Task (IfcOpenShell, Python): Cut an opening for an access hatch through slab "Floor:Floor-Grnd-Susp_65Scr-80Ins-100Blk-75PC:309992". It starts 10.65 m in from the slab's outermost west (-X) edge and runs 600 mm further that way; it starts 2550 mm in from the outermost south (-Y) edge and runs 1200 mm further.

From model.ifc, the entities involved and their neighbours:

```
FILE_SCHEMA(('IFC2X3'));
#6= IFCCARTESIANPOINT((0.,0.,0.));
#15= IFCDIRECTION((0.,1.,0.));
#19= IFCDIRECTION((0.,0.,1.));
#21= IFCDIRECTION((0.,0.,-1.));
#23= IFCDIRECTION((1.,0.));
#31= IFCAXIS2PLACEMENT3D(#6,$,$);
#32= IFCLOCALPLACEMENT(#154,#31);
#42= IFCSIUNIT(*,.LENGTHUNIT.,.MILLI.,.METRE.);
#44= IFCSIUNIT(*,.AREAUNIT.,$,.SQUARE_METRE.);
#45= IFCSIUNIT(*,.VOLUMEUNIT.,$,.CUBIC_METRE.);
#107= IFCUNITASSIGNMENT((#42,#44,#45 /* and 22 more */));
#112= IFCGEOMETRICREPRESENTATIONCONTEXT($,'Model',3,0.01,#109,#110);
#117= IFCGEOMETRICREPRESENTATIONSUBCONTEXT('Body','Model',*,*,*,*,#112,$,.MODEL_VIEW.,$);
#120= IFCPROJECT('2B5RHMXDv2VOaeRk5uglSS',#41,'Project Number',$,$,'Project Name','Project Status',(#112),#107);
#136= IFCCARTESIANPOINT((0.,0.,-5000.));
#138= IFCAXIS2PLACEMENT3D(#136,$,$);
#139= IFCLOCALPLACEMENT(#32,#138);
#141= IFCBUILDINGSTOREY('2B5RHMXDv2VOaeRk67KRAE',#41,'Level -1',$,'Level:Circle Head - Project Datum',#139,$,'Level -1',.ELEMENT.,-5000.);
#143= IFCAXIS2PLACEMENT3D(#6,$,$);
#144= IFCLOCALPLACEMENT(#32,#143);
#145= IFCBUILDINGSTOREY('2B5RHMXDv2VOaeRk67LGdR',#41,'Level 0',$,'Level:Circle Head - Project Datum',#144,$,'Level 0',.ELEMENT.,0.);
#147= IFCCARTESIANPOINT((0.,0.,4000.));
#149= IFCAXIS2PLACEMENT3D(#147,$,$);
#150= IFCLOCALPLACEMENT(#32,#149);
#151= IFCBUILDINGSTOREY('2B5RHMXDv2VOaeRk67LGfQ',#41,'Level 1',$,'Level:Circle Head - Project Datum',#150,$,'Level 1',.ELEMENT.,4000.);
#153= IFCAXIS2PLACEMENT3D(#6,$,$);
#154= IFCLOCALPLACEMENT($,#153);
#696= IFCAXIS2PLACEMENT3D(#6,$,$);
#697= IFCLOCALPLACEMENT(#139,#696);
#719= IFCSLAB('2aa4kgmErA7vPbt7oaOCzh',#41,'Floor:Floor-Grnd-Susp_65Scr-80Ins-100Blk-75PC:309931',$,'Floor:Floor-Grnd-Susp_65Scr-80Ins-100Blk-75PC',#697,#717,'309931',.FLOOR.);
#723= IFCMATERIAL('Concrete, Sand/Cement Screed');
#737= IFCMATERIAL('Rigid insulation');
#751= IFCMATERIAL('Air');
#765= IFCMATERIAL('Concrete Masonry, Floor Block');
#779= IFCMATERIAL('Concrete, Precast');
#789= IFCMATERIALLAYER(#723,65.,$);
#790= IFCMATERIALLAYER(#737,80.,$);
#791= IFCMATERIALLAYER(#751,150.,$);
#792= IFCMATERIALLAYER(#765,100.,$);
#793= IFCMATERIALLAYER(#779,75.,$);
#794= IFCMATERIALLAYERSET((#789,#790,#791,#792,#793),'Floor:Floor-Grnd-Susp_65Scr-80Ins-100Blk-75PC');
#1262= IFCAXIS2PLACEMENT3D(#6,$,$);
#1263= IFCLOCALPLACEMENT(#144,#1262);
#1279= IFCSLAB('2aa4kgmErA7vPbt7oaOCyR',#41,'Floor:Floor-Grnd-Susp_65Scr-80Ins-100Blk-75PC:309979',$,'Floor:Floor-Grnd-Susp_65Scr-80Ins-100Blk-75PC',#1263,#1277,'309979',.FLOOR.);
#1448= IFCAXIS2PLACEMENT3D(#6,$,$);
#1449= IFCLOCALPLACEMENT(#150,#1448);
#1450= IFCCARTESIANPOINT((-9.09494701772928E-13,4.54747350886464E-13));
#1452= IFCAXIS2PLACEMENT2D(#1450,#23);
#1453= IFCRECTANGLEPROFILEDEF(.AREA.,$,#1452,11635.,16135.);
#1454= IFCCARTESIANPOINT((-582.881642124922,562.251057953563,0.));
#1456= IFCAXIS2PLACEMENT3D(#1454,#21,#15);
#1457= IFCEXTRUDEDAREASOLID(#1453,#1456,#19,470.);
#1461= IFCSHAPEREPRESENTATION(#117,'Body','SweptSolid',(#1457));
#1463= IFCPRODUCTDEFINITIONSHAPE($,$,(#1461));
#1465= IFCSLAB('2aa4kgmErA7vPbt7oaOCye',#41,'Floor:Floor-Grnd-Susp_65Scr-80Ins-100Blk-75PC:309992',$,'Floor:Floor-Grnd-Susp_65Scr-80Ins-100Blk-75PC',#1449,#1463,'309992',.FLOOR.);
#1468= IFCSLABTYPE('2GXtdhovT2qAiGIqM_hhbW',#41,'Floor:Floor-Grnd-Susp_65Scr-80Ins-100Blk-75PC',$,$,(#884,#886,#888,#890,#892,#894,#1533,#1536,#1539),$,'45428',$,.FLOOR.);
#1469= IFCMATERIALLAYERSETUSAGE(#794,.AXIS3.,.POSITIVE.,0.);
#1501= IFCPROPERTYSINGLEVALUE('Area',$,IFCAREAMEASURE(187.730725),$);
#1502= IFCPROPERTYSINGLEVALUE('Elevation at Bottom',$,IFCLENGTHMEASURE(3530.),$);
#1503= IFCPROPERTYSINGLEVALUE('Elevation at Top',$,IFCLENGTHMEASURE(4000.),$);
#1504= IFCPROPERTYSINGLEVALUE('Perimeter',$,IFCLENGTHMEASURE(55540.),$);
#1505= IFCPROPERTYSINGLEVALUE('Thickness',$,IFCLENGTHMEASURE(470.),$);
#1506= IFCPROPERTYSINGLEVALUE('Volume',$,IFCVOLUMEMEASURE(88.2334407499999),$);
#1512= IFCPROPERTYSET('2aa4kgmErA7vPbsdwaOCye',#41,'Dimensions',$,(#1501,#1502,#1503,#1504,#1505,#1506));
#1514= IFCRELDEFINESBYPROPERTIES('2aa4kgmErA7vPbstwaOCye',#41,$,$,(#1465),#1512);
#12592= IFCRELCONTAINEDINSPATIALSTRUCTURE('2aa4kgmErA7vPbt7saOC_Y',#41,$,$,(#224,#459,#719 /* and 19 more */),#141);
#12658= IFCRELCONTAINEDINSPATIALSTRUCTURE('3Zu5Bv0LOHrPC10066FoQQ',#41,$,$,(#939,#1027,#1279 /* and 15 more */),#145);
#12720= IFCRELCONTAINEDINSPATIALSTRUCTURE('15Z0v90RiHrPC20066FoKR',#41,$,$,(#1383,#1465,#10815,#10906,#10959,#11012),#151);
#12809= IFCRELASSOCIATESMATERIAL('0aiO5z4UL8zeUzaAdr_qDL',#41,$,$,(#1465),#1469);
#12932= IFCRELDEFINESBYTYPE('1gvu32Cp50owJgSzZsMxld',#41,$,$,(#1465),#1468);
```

```python
import numpy as np
import ifcopenshell
import ifcopenshell.api.feature
import ifcopenshell.api.geometry
import ifcopenshell.api.pset
import ifcopenshell.api.root
import ifcopenshell.geom
import ifcopenshell.util.element
import ifcopenshell.util.placement
import ifcopenshell.util.representation
import ifcopenshell.util.shape
import ifcopenshell.util.unit

model = ifcopenshell.open("model.ifc")
unit_scale = ifcopenshell.util.unit.calculate_unit_scale(model)
area_scale = ifcopenshell.util.unit.calculate_unit_scale(model, "AREAUNIT")
volume_scale = ifcopenshell.util.unit.calculate_unit_scale(model, "VOLUMEUNIT")
settings = ifcopenshell.geom.settings()


def volume(element):
    """Net volume in cubic metres, openings subtracted."""
    shape = ifcopenshell.geom.create_shape(settings, element)
    return ifcopenshell.util.shape.get_volume(shape.geometry)


slab = model.by_guid("2aa4kgmErA7vPbt7oaOCye")
before = volume(slab)

# Extent in the slab's own axes, in metres. The edges named are its -X and -Y sides.
slab_shape = ifcopenshell.geom.create_shape(settings, slab)
vertices = ifcopenshell.util.shape.get_vertices(slab_shape.geometry)
x_min, y_min, bottom = vertices.min(axis=0)
top = vertices[:, 2].max()

opening = ifcopenshell.api.root.create_entity(model, ifc_class="IfcOpeningElement", name="Access hatch opening")
context = ifcopenshell.util.representation.get_context(model, "Model", "Body", "MODEL_VIEW")
width, depth = 0.6, 1.2
outline = [(0.0, 0.0), (width, 0.0), (width, depth), (0.0, depth), (0.0, 0.0)]
# Overshoot both faces by 50 mm so the cut is clean.
shape = ifcopenshell.api.geometry.add_slab_representation(
    model, context=context, depth=top - bottom + 0.1, polyline=outline
)
ifcopenshell.api.geometry.assign_representation(model, product=opening, representation=shape)

matrix = ifcopenshell.util.placement.get_local_placement(slab.ObjectPlacement)
matrix[:, 3] = matrix @ np.append(np.array([x_min + 10.65, y_min + 2.55, bottom - 0.05]) / unit_scale, 1.0)
ifcopenshell.api.geometry.edit_object_placement(model, product=opening, matrix=matrix, is_si=False)
ifcopenshell.api.feature.add_feature(model, feature=opening, element=slab)

after = volume(slab)

# Update the slab's stored quantities.
pset = model.by_id(ifcopenshell.util.element.get_pset(slab, "Dimensions", should_inherit=False)["id"])
ifcopenshell.api.pset.edit_pset(model, pset=pset, properties={
    "Area": model.create_entity("IfcAreaMeasure", after / (top - bottom) / area_scale),
    "Volume": model.create_entity("IfcVolumeMeasure", after / volume_scale),
})

print(f"slab volume {before:.3f} -> {after:.3f} m3")

model.write("model_updated.ifc")
```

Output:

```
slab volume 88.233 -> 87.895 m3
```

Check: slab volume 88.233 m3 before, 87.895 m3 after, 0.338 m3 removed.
